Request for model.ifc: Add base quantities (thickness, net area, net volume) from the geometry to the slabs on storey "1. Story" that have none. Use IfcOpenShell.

First a look at what the model holds.

```python
import ifcopenshell
import ifcopenshell.util.element
import ifcopenshell.util.unit

model = ifcopenshell.open("model.ifc")
print(model.schema)
for unit_type in ("LENGTHUNIT", "AREAUNIT", "VOLUMEUNIT"):
    print(unit_type, ifcopenshell.util.unit.calculate_unit_scale(model, unit_type))
storey = next(s for s in model.by_type("IfcBuildingStorey") if s.Name == "1. Story")
slabs = [e for e in ifcopenshell.util.element.get_decomposition(storey) if e.is_a("IfcSlab")]
for e in sorted(slabs, key=lambda e: e.id()):
    print(e.id(), e.is_a(), e.Name, list(ifcopenshell.util.element.get_psets(e, qtos_only=True)), sep=" | ")
```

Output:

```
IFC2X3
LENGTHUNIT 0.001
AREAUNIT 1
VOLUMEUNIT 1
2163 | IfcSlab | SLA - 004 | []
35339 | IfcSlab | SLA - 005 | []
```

```python
import ifcopenshell
import ifcopenshell.api.pset
import ifcopenshell.geom
import ifcopenshell.util.element
import ifcopenshell.util.shape
import ifcopenshell.util.unit

model = ifcopenshell.open("model.ifc")
unit_scale = ifcopenshell.util.unit.calculate_unit_scale(model)
area_scale = ifcopenshell.util.unit.calculate_unit_scale(model, "AREAUNIT")
volume_scale = ifcopenshell.util.unit.calculate_unit_scale(model, "VOLUMEUNIT")
settings = ifcopenshell.geom.settings()

storey = next(s for s in model.by_type("IfcBuildingStorey") if s.Name == "1. Story")
slabs = [e for e in ifcopenshell.util.element.get_decomposition(storey) if e.is_a("IfcSlab")]

for e in sorted(slabs, key=lambda e: e.id()):
    if ifcopenshell.util.element.get_psets(e, qtos_only=True, should_inherit=False):
        continue
    # Geometry comes back in metres, in the element's own axes.
    shape = ifcopenshell.geom.create_shape(settings, e)
    values = {
        "Width": ifcopenshell.util.shape.get_z(shape.geometry) / unit_scale,
        "NetArea": ifcopenshell.util.shape.get_footprint_area(shape.geometry) / area_scale,
        "NetVolume": ifcopenshell.util.shape.get_volume(shape.geometry) / volume_scale,
    }
    qto = ifcopenshell.api.pset.add_qto(model, product=e, name="BaseQuantities")
    ifcopenshell.api.pset.edit_qto(model, qto=qto, properties=values)
    print(e.id(), {k: round(v, 3) for k, v in values.items()})

model.write("model_rev.ifc")
```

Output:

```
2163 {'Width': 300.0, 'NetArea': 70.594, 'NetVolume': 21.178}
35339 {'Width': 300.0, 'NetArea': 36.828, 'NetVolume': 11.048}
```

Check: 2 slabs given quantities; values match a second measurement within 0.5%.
